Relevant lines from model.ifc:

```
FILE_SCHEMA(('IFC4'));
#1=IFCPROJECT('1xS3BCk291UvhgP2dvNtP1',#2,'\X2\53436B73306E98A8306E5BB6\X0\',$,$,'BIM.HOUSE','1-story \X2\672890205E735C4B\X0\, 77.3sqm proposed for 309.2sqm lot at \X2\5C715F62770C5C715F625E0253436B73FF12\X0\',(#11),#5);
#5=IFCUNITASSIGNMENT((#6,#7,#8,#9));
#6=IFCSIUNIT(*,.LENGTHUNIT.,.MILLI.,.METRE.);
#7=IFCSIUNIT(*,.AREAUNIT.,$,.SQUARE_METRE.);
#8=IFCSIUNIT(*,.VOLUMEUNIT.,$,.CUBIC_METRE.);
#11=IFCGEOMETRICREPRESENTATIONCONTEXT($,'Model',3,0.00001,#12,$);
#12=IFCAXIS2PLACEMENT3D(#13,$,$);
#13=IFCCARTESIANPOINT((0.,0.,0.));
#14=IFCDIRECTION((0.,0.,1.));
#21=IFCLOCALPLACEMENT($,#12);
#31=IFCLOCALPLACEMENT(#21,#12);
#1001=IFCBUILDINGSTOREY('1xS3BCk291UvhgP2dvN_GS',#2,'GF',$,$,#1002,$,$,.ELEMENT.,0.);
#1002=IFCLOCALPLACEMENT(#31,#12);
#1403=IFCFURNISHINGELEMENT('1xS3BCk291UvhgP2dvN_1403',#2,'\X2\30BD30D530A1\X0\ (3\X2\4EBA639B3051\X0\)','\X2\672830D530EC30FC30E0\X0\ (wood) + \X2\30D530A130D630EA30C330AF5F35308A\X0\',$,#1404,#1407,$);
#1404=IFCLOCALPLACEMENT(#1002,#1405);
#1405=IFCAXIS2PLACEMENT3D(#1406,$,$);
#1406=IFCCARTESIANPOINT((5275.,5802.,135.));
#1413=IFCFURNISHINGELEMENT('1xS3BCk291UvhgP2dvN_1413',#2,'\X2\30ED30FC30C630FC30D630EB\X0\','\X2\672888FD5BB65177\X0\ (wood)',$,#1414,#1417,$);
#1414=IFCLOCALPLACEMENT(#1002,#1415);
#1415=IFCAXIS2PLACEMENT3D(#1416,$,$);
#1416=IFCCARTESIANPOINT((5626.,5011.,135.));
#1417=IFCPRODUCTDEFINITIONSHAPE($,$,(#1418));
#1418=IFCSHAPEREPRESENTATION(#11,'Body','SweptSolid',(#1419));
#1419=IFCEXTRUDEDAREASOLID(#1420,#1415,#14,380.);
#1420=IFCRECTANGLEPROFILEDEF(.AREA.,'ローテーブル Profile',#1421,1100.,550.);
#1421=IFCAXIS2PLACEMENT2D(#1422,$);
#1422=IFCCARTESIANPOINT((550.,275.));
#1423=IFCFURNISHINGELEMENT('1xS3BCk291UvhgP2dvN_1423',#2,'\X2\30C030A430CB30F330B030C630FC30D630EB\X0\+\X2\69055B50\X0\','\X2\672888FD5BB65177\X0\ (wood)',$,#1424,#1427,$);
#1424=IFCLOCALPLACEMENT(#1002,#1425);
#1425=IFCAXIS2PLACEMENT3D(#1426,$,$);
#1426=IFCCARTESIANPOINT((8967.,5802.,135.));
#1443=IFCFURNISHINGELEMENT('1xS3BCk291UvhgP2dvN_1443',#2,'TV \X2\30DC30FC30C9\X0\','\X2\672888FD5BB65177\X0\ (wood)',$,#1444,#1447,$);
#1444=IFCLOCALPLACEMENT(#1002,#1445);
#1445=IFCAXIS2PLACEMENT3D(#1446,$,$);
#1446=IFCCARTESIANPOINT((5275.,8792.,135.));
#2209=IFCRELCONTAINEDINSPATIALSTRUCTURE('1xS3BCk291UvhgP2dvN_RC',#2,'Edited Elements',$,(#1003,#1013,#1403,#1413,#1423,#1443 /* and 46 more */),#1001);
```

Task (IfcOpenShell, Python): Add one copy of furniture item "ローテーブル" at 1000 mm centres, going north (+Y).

```python
import numpy as np
import ifcopenshell
import ifcopenshell.api.geometry
import ifcopenshell.api.root
import ifcopenshell.util.element
import ifcopenshell.util.placement
import ifcopenshell.util.unit

model = ifcopenshell.open("model.ifc")
unit_scale = ifcopenshell.util.unit.calculate_unit_scale(model)


def reuse_history(source, copy):
    """copy_class also copies each property set's owner history, people and application; keep the originals."""
    for rel in copy.IsDefinedBy:
        if rel.is_a("IfcRelDefinesByProperties") and (history := rel.RelatingPropertyDefinition.OwnerHistory):
            rel.RelatingPropertyDefinition.OwnerHistory = source.OwnerHistory
            ifcopenshell.util.element.remove_deep2(model, history)


source = model.by_guid("1xS3BCk291UvhgP2dvN_1413")
base = ifcopenshell.util.placement.get_local_placement(source.ObjectPlacement)
step = np.array([0.0, 1.0, 0.0]) * 1 / unit_scale

for i in range(1, 2):
    copy = ifcopenshell.api.root.copy_class(model, product=source)
    copy.Representation = ifcopenshell.util.element.copy_deep(
        model, source.Representation, exclude=["IfcGeometricRepresentationContext", "IfcRepresentationMap"]
    )
    reuse_history(source, copy)
    matrix = base.copy()
    matrix[:3, 3] += i * step
    print("added at", matrix[:3, 3].round(3) + 0.0)
    ifcopenshell.api.geometry.edit_object_placement(model, product=copy, matrix=matrix, is_si=False)

model.write("model_rev.ifc")
```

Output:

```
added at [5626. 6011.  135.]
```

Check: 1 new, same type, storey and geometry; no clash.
